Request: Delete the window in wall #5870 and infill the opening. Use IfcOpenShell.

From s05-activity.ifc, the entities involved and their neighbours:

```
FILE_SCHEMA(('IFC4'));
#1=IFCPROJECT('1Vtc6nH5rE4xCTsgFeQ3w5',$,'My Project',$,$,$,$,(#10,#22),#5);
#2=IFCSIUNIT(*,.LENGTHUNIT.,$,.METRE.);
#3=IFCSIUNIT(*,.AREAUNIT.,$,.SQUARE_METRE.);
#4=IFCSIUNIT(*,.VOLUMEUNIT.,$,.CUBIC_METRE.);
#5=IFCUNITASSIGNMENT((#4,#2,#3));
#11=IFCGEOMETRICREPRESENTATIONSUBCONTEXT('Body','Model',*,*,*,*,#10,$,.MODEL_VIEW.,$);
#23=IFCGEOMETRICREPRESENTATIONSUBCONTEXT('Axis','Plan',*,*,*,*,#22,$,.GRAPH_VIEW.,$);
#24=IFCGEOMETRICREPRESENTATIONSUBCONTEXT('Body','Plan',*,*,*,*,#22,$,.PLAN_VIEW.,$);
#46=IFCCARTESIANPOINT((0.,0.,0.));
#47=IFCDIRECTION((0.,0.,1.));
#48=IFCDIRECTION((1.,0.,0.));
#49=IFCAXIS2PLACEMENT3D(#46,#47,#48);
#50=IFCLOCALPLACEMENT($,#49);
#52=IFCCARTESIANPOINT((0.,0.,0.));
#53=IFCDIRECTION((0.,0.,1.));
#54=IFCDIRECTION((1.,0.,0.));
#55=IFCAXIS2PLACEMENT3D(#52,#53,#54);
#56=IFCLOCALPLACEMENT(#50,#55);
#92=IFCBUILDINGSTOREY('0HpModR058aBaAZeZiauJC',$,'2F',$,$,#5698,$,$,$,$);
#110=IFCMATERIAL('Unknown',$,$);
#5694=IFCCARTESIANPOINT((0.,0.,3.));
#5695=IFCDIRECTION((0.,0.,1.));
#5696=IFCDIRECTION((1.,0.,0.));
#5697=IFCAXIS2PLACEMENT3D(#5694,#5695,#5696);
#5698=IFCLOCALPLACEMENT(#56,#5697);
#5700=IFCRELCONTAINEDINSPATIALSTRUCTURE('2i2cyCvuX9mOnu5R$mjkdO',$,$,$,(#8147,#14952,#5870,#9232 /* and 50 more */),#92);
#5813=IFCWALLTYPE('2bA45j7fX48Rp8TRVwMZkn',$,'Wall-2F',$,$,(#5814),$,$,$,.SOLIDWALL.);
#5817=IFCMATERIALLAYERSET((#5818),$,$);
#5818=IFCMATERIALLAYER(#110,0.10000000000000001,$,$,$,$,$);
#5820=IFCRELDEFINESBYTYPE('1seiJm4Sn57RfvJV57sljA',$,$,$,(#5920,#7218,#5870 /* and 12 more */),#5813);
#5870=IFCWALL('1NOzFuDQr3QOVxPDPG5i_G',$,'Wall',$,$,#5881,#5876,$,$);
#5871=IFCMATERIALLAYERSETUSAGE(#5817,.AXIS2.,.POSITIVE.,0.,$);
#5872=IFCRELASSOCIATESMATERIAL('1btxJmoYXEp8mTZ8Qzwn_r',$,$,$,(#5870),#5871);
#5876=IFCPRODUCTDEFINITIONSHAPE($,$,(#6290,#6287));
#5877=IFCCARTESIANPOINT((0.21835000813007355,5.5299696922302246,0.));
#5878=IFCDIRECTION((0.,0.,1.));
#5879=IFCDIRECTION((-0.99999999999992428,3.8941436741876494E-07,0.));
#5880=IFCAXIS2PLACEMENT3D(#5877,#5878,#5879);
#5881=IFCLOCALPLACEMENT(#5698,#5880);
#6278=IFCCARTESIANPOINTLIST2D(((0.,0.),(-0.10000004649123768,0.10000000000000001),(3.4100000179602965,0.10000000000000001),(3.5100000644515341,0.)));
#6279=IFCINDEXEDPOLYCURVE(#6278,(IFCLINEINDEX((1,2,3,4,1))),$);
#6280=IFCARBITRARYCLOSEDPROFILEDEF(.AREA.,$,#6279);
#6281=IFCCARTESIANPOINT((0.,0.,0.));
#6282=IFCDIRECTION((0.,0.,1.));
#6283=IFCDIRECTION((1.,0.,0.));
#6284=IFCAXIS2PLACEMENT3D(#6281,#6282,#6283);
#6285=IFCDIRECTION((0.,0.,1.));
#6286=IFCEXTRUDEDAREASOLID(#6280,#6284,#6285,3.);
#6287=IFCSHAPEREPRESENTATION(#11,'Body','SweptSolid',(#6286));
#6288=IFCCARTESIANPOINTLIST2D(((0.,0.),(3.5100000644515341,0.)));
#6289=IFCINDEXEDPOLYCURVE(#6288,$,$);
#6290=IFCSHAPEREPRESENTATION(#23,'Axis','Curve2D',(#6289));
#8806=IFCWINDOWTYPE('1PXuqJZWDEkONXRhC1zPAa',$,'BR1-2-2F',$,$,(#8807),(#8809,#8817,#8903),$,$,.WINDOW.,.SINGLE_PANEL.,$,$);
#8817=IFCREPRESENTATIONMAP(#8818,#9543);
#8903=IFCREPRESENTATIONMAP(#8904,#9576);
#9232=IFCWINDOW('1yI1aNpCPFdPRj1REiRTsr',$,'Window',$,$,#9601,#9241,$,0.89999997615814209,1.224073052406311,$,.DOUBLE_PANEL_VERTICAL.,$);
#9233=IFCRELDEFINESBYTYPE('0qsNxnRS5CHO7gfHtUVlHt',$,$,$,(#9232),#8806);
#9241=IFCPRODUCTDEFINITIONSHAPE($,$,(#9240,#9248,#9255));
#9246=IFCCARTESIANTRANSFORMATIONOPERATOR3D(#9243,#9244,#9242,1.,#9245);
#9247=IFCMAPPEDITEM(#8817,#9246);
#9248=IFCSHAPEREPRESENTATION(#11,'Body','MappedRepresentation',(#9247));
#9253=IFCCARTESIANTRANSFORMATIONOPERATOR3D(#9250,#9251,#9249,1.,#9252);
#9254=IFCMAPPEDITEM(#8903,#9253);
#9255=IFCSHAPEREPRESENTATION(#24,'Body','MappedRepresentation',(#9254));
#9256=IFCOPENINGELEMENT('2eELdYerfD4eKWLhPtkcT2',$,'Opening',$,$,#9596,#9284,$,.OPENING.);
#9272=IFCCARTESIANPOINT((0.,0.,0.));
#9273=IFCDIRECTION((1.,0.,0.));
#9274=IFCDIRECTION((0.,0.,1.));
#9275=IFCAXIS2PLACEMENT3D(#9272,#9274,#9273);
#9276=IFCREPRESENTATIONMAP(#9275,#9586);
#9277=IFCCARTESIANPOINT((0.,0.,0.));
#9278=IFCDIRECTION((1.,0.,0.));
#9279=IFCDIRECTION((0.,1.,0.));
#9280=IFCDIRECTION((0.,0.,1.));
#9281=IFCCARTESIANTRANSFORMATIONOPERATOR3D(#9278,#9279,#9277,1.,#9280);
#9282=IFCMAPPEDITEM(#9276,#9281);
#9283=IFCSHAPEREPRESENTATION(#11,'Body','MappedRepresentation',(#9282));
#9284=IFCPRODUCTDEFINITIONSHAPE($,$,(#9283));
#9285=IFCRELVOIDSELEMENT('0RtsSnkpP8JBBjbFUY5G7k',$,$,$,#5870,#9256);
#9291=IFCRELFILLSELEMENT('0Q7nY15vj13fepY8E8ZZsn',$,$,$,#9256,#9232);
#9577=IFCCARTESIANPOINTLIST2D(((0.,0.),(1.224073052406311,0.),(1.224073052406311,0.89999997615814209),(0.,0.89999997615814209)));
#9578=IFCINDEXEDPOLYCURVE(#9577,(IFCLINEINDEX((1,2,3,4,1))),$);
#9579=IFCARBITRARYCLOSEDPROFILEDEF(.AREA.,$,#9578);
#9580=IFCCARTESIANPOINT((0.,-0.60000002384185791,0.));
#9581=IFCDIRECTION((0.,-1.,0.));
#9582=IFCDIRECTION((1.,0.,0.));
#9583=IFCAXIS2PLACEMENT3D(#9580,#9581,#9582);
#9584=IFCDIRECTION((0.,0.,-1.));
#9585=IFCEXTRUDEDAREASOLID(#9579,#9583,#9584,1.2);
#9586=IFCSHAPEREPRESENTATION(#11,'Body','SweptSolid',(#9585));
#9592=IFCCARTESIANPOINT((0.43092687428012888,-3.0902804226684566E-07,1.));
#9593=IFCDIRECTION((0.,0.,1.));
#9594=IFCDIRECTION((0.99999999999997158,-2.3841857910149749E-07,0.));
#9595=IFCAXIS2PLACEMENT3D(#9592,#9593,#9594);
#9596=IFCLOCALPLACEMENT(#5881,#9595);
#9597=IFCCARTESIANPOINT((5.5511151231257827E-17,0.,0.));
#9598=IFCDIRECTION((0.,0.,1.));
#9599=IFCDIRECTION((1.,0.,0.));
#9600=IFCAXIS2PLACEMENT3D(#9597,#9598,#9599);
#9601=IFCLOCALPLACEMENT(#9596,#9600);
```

```python
import ifcopenshell
import ifcopenshell.api.feature
import ifcopenshell.api.root
import ifcopenshell.geom
import ifcopenshell.util.shape

model = ifcopenshell.open("s05-activity.ifc")
settings = ifcopenshell.geom.settings()


def volume(element):
    """Net volume in cubic metres, openings subtracted."""
    shape = ifcopenshell.geom.create_shape(settings, element)
    return ifcopenshell.util.shape.get_volume(shape.geometry)


window = model.by_guid("1yI1aNpCPFdPRj1REiRTsr")
opening = window.FillsVoids[0].RelatingOpeningElement
wall = opening.VoidsElements[0].RelatingBuildingElement
before = volume(wall)

ifcopenshell.api.root.remove_product(model, product=window)
ifcopenshell.api.feature.remove_feature(model, feature=opening)

after = volume(wall)

print(f"wall volume {before:.3f} -> {after:.3f} m3")

model.write("s05-activity_edited.ifc")
```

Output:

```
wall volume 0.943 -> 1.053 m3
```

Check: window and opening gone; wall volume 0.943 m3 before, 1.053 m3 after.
